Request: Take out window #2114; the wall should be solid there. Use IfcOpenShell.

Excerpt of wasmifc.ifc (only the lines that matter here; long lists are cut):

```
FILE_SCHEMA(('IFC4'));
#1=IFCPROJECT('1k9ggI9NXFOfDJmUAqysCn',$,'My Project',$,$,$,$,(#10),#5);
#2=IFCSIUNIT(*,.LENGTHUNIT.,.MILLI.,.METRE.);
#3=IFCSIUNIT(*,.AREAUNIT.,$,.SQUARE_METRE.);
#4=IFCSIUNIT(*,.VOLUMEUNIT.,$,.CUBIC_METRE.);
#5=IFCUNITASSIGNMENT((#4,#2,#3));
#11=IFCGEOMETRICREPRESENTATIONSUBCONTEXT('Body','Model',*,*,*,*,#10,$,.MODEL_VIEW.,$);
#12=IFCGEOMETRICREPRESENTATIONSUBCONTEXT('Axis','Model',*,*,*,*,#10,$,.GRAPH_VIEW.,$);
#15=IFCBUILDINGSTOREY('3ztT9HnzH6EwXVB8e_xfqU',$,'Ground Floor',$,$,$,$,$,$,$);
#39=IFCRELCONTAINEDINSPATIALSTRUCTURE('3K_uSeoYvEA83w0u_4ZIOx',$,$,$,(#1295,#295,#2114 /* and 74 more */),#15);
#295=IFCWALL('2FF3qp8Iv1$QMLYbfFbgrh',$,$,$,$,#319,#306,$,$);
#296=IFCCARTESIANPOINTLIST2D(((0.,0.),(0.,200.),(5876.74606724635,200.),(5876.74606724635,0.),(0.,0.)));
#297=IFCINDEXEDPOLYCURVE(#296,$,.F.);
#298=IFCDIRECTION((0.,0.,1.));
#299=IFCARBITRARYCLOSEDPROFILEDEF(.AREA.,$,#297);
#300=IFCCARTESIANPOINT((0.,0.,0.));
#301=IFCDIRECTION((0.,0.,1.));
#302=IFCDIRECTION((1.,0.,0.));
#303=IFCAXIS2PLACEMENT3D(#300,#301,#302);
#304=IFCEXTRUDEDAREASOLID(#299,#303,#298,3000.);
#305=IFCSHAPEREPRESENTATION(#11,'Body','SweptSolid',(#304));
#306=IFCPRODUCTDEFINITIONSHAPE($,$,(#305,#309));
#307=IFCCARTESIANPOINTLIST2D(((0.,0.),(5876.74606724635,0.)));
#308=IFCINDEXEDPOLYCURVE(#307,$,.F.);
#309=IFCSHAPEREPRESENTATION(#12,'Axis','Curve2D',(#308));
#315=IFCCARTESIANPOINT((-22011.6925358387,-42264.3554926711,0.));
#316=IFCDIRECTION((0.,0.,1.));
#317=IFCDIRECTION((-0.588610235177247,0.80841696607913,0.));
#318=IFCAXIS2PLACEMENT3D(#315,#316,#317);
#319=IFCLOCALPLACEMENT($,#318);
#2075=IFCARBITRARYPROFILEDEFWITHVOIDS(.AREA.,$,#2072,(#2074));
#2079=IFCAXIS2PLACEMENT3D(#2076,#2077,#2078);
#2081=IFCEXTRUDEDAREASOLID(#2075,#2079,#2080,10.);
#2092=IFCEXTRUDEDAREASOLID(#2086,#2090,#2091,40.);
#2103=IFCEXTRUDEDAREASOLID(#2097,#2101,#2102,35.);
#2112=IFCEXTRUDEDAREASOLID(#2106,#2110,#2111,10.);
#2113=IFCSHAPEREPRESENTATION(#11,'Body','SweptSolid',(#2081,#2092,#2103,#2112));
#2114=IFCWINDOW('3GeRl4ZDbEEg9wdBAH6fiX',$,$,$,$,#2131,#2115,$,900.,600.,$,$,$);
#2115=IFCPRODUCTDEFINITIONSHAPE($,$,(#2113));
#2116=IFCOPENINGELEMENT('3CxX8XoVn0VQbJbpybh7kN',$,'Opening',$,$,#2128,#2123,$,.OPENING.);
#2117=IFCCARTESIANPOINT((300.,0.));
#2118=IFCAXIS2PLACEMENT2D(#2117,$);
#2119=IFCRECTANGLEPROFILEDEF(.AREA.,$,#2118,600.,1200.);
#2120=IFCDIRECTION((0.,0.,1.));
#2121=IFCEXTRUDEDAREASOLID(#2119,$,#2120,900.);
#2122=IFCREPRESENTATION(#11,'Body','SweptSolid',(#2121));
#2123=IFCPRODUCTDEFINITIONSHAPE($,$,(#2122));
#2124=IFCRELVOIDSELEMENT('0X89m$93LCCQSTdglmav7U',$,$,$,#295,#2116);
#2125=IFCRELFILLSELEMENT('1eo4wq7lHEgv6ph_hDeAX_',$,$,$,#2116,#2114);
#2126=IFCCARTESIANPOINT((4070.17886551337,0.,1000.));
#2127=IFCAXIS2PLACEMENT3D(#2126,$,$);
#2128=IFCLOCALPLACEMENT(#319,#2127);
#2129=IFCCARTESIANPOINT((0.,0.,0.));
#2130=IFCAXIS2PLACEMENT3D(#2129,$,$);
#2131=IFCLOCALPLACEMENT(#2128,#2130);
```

```python
import ifcopenshell
import ifcopenshell.api.feature
import ifcopenshell.api.root
import ifcopenshell.geom
import ifcopenshell.util.shape

model = ifcopenshell.open("wasmifc.ifc")
settings = ifcopenshell.geom.settings()


def volume(element):
    """Net volume in cubic metres, openings subtracted."""
    shape = ifcopenshell.geom.create_shape(settings, element)
    return ifcopenshell.util.shape.get_volume(shape.geometry)


window = model.by_guid("3GeRl4ZDbEEg9wdBAH6fiX")
opening = window.FillsVoids[0].RelatingOpeningElement
wall = opening.VoidsElements[0].RelatingBuildingElement
before = volume(wall)

ifcopenshell.api.root.remove_product(model, product=window)
ifcopenshell.api.feature.remove_feature(model, feature=opening)

after = volume(wall)

print(f"wall volume {before:.3f} -> {after:.3f} m3")

model.write("wasmifc_v2.ifc")
```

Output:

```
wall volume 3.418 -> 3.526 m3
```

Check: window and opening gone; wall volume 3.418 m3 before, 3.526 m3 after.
